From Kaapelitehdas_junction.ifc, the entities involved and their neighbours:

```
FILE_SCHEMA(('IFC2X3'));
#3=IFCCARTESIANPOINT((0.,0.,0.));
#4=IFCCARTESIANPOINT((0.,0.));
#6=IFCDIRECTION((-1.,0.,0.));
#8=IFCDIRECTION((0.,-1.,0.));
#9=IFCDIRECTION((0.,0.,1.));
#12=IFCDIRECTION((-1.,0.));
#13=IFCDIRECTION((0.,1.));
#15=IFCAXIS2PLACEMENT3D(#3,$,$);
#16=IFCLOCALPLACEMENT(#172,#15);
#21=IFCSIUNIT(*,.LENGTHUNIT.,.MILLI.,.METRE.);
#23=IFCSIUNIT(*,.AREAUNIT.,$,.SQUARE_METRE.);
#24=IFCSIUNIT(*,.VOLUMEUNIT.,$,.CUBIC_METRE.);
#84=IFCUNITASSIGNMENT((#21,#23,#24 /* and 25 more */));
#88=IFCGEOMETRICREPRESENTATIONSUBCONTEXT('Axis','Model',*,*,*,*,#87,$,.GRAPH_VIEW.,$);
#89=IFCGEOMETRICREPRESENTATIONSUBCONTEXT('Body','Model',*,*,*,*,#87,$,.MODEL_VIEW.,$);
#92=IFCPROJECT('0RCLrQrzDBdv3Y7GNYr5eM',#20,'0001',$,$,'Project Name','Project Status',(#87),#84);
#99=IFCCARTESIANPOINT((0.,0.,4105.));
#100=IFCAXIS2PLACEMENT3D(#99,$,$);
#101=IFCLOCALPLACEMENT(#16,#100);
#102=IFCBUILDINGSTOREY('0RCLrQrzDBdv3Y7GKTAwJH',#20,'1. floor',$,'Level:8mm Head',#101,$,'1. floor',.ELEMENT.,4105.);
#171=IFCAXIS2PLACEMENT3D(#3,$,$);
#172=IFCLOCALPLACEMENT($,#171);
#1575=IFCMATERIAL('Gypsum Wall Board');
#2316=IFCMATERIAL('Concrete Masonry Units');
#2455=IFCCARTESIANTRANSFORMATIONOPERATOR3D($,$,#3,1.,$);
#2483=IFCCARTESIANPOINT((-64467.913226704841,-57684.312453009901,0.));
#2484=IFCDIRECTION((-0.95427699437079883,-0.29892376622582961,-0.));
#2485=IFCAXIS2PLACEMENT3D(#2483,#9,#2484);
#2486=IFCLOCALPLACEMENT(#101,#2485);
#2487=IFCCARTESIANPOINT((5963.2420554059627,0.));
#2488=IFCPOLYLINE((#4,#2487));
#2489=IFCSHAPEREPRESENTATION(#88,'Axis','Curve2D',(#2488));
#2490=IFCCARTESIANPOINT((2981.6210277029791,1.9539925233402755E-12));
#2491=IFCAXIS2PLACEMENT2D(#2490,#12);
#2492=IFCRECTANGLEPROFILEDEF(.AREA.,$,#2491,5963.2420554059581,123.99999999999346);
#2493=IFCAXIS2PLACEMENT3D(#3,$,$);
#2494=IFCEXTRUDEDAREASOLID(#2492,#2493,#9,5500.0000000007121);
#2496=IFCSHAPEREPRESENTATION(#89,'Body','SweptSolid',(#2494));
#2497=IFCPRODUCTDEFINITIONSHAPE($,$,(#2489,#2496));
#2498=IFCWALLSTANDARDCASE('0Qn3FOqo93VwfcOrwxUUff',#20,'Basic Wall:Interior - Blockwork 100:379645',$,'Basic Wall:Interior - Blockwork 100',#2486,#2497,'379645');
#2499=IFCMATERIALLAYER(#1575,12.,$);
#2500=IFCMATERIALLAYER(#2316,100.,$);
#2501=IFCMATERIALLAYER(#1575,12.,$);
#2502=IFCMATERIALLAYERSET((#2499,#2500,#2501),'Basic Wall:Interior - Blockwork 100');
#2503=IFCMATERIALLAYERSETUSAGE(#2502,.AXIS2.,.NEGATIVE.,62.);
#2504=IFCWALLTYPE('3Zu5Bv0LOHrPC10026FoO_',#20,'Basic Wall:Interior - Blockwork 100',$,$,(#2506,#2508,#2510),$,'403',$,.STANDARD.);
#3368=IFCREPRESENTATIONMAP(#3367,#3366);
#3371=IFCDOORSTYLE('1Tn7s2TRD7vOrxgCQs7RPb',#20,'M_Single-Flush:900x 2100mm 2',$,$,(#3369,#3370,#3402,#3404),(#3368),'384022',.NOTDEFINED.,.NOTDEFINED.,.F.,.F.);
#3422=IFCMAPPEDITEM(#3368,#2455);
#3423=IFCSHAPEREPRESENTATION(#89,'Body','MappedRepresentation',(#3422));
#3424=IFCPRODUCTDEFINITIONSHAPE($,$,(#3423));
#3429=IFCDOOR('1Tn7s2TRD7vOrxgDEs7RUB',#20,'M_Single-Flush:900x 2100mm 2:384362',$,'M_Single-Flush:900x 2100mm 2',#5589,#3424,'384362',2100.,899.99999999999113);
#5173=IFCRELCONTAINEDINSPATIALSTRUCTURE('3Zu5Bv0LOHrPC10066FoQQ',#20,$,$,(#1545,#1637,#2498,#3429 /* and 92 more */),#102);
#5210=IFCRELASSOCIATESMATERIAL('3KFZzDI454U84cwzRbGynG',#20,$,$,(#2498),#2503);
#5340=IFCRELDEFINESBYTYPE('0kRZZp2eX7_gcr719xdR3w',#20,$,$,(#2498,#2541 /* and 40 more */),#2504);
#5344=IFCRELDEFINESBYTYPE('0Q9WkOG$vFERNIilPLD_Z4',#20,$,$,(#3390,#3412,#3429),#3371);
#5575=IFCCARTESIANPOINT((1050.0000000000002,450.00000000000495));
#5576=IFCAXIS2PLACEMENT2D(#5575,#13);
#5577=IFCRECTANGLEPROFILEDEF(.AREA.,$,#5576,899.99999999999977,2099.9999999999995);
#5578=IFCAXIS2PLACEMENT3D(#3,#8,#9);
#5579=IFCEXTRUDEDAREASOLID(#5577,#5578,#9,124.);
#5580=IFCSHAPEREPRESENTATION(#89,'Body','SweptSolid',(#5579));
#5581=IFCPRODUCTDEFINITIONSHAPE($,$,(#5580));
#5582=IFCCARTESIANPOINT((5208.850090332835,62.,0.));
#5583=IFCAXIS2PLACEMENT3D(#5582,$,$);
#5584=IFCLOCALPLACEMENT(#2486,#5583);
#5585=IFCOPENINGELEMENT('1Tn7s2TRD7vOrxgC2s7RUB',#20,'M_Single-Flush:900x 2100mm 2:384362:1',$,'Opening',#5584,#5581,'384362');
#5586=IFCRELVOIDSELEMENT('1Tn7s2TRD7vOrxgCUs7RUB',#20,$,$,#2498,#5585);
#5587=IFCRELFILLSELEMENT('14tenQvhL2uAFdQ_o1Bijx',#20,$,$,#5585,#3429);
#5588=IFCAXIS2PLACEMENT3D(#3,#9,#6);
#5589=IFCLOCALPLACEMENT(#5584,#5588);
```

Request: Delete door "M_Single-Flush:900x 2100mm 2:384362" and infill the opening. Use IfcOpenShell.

```python
import ifcopenshell
import ifcopenshell.api.feature
import ifcopenshell.api.root
import ifcopenshell.geom
import ifcopenshell.util.shape

model = ifcopenshell.open("Kaapelitehdas_junction.ifc")
settings = ifcopenshell.geom.settings()


def volume(element):
    """Net volume in cubic metres, openings subtracted."""
    shape = ifcopenshell.geom.create_shape(settings, element)
    return ifcopenshell.util.shape.get_volume(shape.geometry)


door = model.by_id(3429)
opening = door.FillsVoids[0].RelatingOpeningElement
wall = opening.VoidsElements[0].RelatingBuildingElement
before = volume(wall)

ifcopenshell.api.root.remove_product(model, product=door)
ifcopenshell.api.feature.remove_feature(model, feature=opening)

after = volume(wall)

print(f"wall volume {before:.3f} -> {after:.3f} m3")

model.write("Kaapelitehdas_junction_v2.ifc")
```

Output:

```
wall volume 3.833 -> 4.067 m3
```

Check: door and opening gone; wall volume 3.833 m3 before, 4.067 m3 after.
